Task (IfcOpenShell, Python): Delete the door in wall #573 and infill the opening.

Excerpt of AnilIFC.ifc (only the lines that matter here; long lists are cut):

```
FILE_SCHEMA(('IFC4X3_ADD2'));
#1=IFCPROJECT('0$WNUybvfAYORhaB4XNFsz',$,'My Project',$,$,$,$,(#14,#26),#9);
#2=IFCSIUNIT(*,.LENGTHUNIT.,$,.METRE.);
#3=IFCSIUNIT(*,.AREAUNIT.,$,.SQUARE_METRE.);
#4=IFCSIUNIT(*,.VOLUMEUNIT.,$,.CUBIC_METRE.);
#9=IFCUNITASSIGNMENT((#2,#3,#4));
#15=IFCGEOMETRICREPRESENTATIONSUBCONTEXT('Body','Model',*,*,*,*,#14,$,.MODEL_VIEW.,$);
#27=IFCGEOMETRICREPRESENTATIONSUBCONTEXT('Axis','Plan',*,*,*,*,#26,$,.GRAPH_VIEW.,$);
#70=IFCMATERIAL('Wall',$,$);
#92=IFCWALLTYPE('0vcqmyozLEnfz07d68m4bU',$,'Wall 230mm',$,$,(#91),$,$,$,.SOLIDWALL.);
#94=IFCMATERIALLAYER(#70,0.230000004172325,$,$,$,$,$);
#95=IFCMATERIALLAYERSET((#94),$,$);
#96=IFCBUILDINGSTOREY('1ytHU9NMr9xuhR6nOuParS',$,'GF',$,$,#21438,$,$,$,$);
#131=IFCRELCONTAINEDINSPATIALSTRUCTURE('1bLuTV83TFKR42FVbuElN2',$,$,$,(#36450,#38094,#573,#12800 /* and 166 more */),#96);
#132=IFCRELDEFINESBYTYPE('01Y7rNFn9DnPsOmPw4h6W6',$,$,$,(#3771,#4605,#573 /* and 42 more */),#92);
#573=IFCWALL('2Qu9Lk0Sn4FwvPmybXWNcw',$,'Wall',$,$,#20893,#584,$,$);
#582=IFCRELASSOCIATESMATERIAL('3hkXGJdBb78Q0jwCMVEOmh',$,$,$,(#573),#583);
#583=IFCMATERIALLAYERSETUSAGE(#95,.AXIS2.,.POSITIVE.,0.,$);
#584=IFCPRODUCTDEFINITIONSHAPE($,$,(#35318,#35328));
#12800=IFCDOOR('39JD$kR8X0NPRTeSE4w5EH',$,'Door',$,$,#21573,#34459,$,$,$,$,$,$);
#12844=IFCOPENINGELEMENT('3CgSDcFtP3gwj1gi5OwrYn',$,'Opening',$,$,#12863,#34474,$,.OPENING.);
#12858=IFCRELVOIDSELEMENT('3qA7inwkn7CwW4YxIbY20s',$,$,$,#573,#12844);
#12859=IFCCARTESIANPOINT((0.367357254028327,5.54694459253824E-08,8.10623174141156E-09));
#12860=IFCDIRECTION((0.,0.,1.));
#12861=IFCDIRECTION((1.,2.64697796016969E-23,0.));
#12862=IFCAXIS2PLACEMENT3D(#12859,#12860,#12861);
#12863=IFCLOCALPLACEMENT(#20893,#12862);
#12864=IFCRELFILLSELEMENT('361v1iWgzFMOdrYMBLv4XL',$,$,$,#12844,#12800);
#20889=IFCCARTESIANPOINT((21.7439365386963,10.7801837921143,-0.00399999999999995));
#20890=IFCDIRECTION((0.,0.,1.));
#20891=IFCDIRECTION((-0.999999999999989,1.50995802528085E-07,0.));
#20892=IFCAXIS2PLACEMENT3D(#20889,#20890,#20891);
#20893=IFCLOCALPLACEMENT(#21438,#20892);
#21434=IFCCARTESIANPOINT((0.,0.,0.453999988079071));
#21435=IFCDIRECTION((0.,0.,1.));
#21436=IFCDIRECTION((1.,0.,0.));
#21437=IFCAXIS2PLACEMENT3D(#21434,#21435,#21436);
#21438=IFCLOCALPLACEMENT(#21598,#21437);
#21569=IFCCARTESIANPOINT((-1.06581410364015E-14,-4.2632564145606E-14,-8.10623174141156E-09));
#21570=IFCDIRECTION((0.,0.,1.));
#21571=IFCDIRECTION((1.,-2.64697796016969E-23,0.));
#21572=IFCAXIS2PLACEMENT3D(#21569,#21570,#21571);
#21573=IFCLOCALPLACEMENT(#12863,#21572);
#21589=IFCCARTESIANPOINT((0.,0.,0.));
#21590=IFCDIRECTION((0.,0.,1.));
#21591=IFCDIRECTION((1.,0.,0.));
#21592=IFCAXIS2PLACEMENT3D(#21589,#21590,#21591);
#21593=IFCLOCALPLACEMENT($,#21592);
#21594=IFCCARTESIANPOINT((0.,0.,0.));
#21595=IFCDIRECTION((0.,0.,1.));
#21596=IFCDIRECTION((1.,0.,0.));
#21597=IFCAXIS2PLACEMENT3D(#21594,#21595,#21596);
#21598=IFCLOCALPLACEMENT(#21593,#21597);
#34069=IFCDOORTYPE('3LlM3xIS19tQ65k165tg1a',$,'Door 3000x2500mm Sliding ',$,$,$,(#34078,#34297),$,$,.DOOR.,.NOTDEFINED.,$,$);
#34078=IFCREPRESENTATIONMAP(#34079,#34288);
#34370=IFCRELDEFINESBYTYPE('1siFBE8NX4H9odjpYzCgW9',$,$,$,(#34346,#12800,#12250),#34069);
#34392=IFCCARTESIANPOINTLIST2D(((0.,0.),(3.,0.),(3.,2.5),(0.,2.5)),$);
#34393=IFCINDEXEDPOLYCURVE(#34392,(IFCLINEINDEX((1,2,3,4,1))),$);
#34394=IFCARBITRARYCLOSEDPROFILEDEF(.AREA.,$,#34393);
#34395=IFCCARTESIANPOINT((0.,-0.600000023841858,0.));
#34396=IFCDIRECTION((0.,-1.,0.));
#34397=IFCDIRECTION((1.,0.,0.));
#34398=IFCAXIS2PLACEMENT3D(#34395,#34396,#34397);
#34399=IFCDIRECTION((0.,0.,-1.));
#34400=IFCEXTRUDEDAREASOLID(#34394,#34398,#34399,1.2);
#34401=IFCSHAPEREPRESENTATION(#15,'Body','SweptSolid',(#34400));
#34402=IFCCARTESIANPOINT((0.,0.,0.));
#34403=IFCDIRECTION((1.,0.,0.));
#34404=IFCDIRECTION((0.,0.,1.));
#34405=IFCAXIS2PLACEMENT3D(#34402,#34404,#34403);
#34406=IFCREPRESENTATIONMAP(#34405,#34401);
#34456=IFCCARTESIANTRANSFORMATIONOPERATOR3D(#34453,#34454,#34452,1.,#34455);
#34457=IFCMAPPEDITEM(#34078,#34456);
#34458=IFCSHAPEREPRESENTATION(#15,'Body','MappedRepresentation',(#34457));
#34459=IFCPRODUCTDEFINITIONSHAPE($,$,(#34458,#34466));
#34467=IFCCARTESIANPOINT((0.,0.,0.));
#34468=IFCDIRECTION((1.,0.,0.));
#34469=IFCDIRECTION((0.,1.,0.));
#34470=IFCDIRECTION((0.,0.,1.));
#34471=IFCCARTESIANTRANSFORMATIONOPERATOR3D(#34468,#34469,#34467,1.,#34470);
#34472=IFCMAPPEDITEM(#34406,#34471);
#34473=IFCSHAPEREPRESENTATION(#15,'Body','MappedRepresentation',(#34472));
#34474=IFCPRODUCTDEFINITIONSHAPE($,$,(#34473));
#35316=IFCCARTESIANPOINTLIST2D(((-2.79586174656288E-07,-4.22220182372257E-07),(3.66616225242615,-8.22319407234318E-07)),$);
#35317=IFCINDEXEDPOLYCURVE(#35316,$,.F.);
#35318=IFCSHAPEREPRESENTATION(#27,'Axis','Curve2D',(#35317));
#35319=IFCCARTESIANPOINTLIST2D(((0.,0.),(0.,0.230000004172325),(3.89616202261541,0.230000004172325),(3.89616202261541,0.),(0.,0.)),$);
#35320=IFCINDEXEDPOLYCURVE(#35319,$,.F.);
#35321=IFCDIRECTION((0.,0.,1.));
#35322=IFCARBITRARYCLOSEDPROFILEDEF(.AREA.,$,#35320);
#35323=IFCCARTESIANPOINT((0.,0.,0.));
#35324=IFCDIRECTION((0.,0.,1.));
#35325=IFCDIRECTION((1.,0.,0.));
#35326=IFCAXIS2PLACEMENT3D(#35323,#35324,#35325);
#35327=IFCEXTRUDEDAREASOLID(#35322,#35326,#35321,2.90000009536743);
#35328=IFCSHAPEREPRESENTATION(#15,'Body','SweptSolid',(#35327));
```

```python
import ifcopenshell
import ifcopenshell.api.feature
import ifcopenshell.api.root
import ifcopenshell.geom
import ifcopenshell.util.shape

model = ifcopenshell.open("AnilIFC.ifc")
settings = ifcopenshell.geom.settings()


def volume(element):
    """Net volume in cubic metres, openings subtracted."""
    shape = ifcopenshell.geom.create_shape(settings, element)
    return ifcopenshell.util.shape.get_volume(shape.geometry)


door = model.by_id(12800)
opening = door.FillsVoids[0].RelatingOpeningElement
wall = opening.VoidsElements[0].RelatingBuildingElement
before = volume(wall)

ifcopenshell.api.root.remove_product(model, product=door)
ifcopenshell.api.feature.remove_feature(model, feature=opening)

after = volume(wall)

print(f"wall volume {before:.3f} -> {after:.3f} m3")

model.write("AnilIFC-out.ifc")
```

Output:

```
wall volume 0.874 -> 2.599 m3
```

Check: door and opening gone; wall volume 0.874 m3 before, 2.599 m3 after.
